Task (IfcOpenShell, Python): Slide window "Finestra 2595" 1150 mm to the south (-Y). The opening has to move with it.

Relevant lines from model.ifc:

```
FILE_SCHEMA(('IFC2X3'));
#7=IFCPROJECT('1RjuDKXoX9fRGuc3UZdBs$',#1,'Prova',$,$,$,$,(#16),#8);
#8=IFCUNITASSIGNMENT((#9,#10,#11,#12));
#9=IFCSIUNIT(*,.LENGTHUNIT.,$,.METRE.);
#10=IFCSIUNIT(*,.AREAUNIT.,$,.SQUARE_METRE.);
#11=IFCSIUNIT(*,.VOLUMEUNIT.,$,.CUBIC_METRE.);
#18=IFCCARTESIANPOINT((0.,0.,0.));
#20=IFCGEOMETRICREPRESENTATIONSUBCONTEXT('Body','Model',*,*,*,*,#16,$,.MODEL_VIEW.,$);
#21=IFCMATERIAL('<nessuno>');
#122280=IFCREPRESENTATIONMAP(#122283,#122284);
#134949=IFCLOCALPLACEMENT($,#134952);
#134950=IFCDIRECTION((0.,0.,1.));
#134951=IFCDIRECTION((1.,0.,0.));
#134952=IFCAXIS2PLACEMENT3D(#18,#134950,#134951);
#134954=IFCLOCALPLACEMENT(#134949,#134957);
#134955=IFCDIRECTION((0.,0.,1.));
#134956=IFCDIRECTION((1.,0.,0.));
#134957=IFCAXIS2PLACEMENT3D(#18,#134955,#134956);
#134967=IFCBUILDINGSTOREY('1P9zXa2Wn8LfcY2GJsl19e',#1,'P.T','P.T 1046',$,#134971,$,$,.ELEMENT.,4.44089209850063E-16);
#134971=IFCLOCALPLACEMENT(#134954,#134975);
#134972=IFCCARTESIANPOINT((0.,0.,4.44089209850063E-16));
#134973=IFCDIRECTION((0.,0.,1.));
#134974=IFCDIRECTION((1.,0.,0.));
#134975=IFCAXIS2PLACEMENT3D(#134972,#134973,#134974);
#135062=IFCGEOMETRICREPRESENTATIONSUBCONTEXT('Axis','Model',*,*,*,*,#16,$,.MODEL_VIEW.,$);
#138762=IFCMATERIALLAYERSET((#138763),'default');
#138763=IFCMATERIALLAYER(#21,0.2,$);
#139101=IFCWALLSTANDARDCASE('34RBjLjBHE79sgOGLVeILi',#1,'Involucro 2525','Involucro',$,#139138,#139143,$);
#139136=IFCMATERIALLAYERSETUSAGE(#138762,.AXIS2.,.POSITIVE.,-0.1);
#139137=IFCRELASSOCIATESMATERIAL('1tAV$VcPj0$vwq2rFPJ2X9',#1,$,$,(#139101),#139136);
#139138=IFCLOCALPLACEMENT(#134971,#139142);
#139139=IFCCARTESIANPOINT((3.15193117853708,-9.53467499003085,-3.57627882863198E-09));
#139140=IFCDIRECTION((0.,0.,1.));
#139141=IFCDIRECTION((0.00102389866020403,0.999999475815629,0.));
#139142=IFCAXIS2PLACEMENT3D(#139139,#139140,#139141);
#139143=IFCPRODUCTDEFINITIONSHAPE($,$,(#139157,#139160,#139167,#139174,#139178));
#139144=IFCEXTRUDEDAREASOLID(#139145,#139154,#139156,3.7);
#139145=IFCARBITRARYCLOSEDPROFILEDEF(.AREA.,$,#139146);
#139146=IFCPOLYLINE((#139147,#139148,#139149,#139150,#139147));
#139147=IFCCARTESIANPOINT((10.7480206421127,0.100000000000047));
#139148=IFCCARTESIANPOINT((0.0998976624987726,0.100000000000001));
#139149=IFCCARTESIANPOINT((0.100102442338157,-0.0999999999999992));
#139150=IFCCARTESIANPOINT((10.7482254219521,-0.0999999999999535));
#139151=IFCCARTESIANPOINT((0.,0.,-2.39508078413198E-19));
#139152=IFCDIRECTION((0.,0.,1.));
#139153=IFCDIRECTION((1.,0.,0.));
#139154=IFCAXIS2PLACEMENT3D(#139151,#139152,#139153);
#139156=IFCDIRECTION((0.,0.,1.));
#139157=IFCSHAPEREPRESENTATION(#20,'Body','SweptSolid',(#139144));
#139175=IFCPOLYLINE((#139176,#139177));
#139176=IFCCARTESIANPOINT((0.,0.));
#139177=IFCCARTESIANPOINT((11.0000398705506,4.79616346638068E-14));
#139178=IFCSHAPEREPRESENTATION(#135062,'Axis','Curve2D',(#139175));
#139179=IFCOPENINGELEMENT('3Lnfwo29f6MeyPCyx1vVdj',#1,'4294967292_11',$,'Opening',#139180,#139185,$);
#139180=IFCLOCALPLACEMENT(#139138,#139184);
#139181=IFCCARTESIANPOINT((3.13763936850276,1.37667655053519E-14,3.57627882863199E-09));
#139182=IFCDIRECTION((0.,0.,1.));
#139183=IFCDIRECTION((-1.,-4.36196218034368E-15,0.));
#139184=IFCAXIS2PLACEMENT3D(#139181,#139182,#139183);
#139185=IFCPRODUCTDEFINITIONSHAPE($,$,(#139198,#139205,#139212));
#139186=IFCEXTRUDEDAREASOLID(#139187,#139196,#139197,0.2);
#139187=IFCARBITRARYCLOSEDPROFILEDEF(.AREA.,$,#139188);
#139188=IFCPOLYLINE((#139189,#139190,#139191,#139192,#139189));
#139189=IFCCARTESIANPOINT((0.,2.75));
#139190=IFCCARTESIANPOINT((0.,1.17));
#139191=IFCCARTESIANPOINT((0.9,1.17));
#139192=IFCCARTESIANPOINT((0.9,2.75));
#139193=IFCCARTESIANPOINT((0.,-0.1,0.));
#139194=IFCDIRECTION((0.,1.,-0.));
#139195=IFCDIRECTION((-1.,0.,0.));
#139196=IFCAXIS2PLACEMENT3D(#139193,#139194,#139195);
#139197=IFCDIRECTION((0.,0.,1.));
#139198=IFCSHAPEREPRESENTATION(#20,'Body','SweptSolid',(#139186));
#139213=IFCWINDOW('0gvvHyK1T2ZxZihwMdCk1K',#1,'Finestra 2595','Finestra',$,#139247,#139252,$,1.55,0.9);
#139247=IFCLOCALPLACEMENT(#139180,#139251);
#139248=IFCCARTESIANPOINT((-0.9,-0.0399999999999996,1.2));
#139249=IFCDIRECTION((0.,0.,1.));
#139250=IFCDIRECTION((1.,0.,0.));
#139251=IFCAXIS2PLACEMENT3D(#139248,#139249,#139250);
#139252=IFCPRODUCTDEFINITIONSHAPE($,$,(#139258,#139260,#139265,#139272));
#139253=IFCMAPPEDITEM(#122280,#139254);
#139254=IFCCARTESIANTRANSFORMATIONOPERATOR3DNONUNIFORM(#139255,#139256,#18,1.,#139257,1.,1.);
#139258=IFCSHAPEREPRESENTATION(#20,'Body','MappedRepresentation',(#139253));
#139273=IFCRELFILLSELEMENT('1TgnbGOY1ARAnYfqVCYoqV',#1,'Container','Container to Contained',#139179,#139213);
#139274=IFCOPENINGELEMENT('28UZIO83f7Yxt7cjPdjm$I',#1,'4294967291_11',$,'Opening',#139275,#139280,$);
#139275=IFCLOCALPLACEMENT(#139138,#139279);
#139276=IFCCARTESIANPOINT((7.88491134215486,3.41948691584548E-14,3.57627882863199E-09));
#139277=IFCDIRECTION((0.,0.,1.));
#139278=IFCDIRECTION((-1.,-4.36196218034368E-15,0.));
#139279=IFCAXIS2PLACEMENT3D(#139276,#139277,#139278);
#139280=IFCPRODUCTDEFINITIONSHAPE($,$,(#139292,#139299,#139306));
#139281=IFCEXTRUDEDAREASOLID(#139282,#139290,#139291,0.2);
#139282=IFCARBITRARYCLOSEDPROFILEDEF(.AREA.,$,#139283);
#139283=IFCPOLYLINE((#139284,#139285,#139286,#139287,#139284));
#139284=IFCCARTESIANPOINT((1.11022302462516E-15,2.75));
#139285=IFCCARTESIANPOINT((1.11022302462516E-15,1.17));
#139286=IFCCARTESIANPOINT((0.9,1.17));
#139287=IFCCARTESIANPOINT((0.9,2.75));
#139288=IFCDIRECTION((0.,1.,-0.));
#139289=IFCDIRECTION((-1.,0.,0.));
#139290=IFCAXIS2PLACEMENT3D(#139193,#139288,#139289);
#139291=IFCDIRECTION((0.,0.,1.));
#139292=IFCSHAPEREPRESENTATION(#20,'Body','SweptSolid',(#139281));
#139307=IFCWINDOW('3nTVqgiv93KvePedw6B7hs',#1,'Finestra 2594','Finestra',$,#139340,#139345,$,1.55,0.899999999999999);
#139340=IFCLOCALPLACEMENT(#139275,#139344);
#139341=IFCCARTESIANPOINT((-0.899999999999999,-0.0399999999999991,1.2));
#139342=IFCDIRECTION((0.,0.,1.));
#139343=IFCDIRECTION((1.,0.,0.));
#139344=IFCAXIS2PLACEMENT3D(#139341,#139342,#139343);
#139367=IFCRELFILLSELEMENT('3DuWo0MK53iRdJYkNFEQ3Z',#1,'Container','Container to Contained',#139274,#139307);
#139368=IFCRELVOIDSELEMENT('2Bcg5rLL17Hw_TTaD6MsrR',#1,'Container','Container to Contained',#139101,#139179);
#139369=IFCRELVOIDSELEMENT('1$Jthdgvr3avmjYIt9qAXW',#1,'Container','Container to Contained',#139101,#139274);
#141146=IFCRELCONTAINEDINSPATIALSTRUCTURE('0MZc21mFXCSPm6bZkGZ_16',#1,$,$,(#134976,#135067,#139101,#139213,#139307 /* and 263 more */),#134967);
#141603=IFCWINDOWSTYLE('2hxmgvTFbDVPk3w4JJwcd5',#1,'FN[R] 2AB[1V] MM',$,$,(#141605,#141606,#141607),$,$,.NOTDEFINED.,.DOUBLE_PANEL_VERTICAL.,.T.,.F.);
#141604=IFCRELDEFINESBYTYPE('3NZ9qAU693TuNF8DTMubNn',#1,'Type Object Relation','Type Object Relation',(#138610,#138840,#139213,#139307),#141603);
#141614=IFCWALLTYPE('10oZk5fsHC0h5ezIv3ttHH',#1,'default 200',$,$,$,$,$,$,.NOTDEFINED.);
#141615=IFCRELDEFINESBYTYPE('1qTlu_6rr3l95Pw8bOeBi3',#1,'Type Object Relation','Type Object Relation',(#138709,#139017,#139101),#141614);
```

```python
import ifcopenshell
import ifcopenshell.api.geometry
import ifcopenshell.util.placement
import ifcopenshell.util.unit

model = ifcopenshell.open("model.ifc")
unit_scale = ifcopenshell.util.unit.calculate_unit_scale(model)

window = model.by_guid("0gvvHyK1T2ZxZihwMdCk1K")
opening = window.FillsVoids[0].RelatingOpeningElement
wall = opening.VoidsElements[0].RelatingBuildingElement

wall_matrix = ifcopenshell.util.placement.get_local_placement(wall.ObjectPlacement)
shift = wall_matrix[:3, 0] * -1.15 / unit_scale
before = ifcopenshell.util.placement.get_local_placement(window.ObjectPlacement)[:3, 3].copy()

# The window is placed relative to its opening, so it follows when the opening moves.
matrix = ifcopenshell.util.placement.get_local_placement(opening.ObjectPlacement)
matrix[:3, 3] += shift
ifcopenshell.api.geometry.edit_object_placement(
    model, product=opening, matrix=matrix, is_si=False, should_transform_children=True
)

after = ifcopenshell.util.placement.get_local_placement(window.ObjectPlacement)[:3, 3]
print("window moved by", (after - before).round(3) + 0.0)

model.write("model-out.ifc")
```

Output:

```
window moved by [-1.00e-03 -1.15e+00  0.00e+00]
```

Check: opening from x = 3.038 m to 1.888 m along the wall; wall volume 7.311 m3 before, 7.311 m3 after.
